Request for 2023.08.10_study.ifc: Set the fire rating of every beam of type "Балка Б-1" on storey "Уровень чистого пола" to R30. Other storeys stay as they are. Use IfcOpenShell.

First a look at what the model holds.

```python
import ifcopenshell
import ifcopenshell.util.element

model = ifcopenshell.open("2023.08.10_study.ifc")
print(model.schema)
storey = next(s for s in model.by_type("IfcBuildingStorey") if s.Name == "Уровень чистого пола")
beams = [e for e in ifcopenshell.util.element.get_decomposition(storey) if e.is_a("IfcBeam")]
seen = {}
for e in beams:
    element_type = ifcopenshell.util.element.get_type(e)
    key = (element_type.Name if element_type != e and element_type else None, ifcopenshell.util.element.get_pset(e, "Pset_BeamCommon", "FireRating"))
    seen[key] = seen.get(key, 0) + 1
for (name, value), count in sorted(seen.items(), key=str):
    print(count, "x", name, "|", value)
```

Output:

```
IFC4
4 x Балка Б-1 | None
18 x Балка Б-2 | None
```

```python
import ifcopenshell
import ifcopenshell.api.pset
import ifcopenshell.util.element

model = ifcopenshell.open("2023.08.10_study.ifc")

storey = next(s for s in model.by_type("IfcBuildingStorey") if s.Name == "Уровень чистого пола")
beams = [e for e in ifcopenshell.util.element.get_decomposition(storey) if e.is_a("IfcBeam")]

count = 0
for e in beams:
    element_type = ifcopenshell.util.element.get_type(e)
    if element_type in (None, e) or element_type.Name != "Балка Б-1":
        continue
    # add_pset returns the element's existing set when there is one.
    pset = ifcopenshell.api.pset.add_pset(model, product=e, name="Pset_BeamCommon")
    ifcopenshell.api.pset.edit_pset(model, pset=pset, properties={"FireRating": "R30"})
    count += 1

print(count, "beams updated")

model.write("2023.08.10_study_edited.ifc")
```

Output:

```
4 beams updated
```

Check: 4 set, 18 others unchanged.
